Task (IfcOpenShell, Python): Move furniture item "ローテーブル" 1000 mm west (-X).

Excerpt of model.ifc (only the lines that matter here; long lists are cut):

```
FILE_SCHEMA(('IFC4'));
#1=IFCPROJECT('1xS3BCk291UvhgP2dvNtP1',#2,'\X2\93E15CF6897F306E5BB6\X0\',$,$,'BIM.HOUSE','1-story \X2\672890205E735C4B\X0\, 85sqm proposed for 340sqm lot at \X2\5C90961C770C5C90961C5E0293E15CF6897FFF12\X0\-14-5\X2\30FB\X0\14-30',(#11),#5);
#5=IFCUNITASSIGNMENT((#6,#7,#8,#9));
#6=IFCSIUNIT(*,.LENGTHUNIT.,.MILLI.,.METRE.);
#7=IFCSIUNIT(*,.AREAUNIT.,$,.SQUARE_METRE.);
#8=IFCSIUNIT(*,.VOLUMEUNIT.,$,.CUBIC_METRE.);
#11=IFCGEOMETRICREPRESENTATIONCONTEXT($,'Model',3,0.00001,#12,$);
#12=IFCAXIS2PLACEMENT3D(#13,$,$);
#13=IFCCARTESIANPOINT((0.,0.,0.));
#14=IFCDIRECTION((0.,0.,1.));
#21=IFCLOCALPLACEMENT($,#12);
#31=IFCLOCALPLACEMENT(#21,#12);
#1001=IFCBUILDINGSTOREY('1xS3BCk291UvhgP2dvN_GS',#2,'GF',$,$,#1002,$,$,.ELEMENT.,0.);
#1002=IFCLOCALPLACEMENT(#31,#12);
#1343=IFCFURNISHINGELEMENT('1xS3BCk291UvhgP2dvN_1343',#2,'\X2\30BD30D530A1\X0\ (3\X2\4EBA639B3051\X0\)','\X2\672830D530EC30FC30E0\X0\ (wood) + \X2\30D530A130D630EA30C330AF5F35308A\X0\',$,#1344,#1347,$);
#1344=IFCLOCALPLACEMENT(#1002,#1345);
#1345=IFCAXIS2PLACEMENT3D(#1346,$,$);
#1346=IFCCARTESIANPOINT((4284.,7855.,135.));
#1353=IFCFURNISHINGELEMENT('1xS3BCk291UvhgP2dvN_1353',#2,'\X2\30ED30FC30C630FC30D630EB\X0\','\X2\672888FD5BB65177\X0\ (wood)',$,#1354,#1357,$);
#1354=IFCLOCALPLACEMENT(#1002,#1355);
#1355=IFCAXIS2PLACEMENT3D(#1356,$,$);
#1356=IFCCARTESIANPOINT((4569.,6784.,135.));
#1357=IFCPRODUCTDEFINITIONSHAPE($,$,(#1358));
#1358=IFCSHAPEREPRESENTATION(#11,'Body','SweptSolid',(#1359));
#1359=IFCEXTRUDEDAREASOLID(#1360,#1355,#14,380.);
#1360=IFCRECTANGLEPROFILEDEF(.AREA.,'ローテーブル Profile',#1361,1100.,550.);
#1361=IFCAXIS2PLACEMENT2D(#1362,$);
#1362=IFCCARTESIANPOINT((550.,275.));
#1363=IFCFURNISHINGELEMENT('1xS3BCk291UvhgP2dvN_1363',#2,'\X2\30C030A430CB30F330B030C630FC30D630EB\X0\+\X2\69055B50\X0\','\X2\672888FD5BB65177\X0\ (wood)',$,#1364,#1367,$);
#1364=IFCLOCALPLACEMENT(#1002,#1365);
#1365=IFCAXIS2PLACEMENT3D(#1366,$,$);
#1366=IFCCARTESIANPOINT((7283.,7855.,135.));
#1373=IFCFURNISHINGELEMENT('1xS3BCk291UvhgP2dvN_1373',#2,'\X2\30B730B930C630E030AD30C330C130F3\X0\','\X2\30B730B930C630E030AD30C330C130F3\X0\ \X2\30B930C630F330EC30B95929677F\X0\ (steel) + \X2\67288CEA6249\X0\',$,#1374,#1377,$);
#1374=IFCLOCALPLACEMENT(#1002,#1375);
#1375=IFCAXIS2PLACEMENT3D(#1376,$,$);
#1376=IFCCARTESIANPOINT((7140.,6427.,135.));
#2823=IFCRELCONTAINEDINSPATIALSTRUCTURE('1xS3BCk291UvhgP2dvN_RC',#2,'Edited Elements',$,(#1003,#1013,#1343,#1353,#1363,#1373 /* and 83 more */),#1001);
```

```python
import ifcopenshell
import ifcopenshell.api.geometry
import ifcopenshell.util.placement
import ifcopenshell.util.unit

model = ifcopenshell.open("model.ifc")
unit_scale = ifcopenshell.util.unit.calculate_unit_scale(model)

item = model.by_guid("1xS3BCk291UvhgP2dvN_1353")
matrix = ifcopenshell.util.placement.get_local_placement(item.ObjectPlacement)
matrix[0, 3] -= 1 / unit_scale
ifcopenshell.api.geometry.edit_object_placement(model, product=item, matrix=matrix, is_si=False)

print(ifcopenshell.util.placement.get_local_placement(item.ObjectPlacement).round(3) + 0.0)

model.write("model_v2.ifc")
```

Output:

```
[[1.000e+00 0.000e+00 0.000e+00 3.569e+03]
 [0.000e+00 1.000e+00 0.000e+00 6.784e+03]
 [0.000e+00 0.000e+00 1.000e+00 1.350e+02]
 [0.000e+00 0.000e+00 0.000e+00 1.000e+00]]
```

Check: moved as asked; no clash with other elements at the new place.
